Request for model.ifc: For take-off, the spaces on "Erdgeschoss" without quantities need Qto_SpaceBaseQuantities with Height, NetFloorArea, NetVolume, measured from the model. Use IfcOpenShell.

First a look at what the model holds.

```python
import ifcopenshell
import ifcopenshell.util.element
import ifcopenshell.util.unit

model = ifcopenshell.open("model.ifc")
print(model.schema)
for unit_type in ("LENGTHUNIT", "AREAUNIT", "VOLUMEUNIT"):
    print(unit_type, ifcopenshell.util.unit.calculate_unit_scale(model, unit_type))
storey = next(s for s in model.by_type("IfcBuildingStorey") if s.Name == "Erdgeschoss")
spaces = [e for e in ifcopenshell.util.element.get_decomposition(storey) if e.is_a("IfcSpace")]
for e in sorted(spaces, key=lambda e: e.id()):
    print(e.id(), e.is_a(), e.Name, list(ifcopenshell.util.element.get_psets(e, qtos_only=True)), sep=" | ")
```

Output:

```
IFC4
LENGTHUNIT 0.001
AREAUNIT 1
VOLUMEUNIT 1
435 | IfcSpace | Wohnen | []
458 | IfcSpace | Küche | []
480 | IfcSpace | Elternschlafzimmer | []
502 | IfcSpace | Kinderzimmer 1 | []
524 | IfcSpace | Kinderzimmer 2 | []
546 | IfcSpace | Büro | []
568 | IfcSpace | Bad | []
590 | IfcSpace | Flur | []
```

```python
import ifcopenshell
import ifcopenshell.api.pset
import ifcopenshell.geom
import ifcopenshell.util.element
import ifcopenshell.util.shape
import ifcopenshell.util.unit

model = ifcopenshell.open("model.ifc")
unit_scale = ifcopenshell.util.unit.calculate_unit_scale(model)
area_scale = ifcopenshell.util.unit.calculate_unit_scale(model, "AREAUNIT")
volume_scale = ifcopenshell.util.unit.calculate_unit_scale(model, "VOLUMEUNIT")
settings = ifcopenshell.geom.settings()

storey = next(s for s in model.by_type("IfcBuildingStorey") if s.Name == "Erdgeschoss")
spaces = [e for e in ifcopenshell.util.element.get_decomposition(storey) if e.is_a("IfcSpace")]

for e in sorted(spaces, key=lambda e: e.id()):
    if ifcopenshell.util.element.get_psets(e, qtos_only=True, should_inherit=False):
        continue
    # Geometry comes back in metres, in the element's own axes.
    shape = ifcopenshell.geom.create_shape(settings, e)
    values = {
        "Height": ifcopenshell.util.shape.get_z(shape.geometry) / unit_scale,
        "NetFloorArea": ifcopenshell.util.shape.get_footprint_area(shape.geometry) / area_scale,
        "NetVolume": ifcopenshell.util.shape.get_volume(shape.geometry) / volume_scale,
    }
    qto = ifcopenshell.api.pset.add_qto(model, product=e, name="Qto_SpaceBaseQuantities")
    ifcopenshell.api.pset.edit_qto(model, qto=qto, properties=values)
    print(e.id(), {k: round(v, 3) for k, v in values.items()})

model.write("model_updated.ifc")
```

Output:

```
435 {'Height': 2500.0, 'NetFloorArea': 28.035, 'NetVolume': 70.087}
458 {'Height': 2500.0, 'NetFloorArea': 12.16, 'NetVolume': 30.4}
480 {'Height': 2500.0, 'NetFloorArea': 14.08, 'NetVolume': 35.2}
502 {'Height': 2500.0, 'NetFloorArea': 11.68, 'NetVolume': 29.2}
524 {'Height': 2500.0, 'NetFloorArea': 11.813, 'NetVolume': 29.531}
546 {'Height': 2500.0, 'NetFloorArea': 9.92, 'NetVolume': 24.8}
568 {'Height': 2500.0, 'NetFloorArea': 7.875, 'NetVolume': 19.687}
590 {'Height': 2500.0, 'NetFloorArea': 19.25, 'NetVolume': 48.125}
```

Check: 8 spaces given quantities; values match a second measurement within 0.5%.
